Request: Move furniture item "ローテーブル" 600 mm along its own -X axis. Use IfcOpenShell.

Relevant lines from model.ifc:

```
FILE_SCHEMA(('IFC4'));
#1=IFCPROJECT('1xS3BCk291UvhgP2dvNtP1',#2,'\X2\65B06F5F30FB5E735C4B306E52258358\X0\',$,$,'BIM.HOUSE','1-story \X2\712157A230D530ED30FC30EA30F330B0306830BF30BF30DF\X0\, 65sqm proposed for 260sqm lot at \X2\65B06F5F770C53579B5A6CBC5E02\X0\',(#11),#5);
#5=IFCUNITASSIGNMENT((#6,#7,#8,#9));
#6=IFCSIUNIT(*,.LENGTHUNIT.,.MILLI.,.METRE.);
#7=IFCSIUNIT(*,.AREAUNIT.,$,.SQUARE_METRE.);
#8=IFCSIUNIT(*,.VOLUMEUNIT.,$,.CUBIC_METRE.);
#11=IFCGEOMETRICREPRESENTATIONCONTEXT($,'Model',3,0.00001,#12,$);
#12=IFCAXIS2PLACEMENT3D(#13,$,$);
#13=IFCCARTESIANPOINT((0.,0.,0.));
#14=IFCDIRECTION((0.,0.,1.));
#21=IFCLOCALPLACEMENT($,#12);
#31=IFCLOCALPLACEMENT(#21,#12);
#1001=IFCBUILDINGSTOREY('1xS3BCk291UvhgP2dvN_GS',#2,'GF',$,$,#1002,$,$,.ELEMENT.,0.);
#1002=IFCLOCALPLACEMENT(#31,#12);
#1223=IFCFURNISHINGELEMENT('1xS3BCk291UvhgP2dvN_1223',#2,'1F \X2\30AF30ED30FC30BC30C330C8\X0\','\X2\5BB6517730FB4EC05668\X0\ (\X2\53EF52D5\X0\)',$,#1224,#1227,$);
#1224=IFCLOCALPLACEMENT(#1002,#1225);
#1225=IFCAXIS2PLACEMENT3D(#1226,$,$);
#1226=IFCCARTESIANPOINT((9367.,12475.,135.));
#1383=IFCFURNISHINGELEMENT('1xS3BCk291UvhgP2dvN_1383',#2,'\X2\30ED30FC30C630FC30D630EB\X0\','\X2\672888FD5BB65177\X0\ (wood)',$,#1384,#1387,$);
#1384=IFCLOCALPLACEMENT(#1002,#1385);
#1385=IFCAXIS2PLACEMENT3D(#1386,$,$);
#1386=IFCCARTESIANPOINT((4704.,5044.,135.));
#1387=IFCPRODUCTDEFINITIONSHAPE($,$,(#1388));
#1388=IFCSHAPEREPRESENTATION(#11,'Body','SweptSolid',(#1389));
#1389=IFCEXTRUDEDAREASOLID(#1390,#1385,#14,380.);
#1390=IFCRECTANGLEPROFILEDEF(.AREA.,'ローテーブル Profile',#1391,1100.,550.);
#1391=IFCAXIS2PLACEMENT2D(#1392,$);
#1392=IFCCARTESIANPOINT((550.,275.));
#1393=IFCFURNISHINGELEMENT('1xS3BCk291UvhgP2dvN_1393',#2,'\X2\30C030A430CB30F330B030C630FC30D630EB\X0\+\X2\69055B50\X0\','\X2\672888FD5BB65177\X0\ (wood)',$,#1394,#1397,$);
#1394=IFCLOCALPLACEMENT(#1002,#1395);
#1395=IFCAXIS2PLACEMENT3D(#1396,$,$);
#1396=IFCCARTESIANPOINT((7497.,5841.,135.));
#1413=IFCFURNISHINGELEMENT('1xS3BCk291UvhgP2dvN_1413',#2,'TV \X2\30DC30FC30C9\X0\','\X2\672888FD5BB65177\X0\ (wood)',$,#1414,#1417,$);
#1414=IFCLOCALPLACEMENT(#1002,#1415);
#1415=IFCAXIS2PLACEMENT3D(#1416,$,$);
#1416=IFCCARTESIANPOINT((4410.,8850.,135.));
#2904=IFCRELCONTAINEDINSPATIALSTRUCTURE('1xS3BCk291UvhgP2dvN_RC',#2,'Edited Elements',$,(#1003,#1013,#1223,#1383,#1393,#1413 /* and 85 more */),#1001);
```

```python
import ifcopenshell
import ifcopenshell.api.geometry
import ifcopenshell.util.placement

model = ifcopenshell.open("model.ifc")

item = model.by_guid("1xS3BCk291UvhgP2dvN_1383")
matrix = ifcopenshell.util.placement.get_local_placement(item.ObjectPlacement)
matrix[:3, 3] -= matrix[:3, 0] * 600.0
ifcopenshell.api.geometry.edit_object_placement(model, product=item, matrix=matrix, is_si=False)

print(ifcopenshell.util.placement.get_local_placement(item.ObjectPlacement).round(3) + 0.0)

model.write("model_edited.ifc")
```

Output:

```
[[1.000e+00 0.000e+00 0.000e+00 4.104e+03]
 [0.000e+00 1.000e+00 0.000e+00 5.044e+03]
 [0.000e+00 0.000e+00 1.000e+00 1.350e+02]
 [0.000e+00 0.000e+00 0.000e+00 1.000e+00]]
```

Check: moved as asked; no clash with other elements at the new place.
